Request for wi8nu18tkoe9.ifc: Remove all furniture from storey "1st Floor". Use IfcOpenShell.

First a look at what the model holds.

```python
import ifcopenshell
import ifcopenshell.util.element

model = ifcopenshell.open("wi8nu18tkoe9.ifc")
print(model.schema)
storey = next(s for s in model.by_type("IfcBuildingStorey") if s.Name == "1st Floor")
furniture = [e for e in ifcopenshell.util.element.get_decomposition(storey) if e.is_a("IfcFurnishingElement")]
seen = {}
for e in furniture:
    element_type = ifcopenshell.util.element.get_type(e)
    name = element_type.Name if element_type not in (None, e) else None
    seen[name] = seen.get(name, 0) + 1
for name, count in sorted(seen.items(), key=str):
    print(count, "x", name)
```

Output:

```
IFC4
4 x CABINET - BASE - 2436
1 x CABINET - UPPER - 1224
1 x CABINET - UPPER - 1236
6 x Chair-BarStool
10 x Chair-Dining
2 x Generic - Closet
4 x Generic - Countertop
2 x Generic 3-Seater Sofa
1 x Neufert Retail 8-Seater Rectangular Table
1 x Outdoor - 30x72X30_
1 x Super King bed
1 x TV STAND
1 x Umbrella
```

```python
import ifcopenshell
import ifcopenshell.api.root
import ifcopenshell.util.element

model = ifcopenshell.open("wi8nu18tkoe9.ifc")

storey = next(s for s in model.by_type("IfcBuildingStorey") if s.Name == "1st Floor")
furniture = [e for e in ifcopenshell.util.element.get_decomposition(storey) if e.is_a("IfcFurnishingElement")]

for e in furniture:
    ifcopenshell.api.root.remove_product(model, product=e)
print(len(furniture), "removed")

model.write("wi8nu18tkoe9_v2.ifc")
```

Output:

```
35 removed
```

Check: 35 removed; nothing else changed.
